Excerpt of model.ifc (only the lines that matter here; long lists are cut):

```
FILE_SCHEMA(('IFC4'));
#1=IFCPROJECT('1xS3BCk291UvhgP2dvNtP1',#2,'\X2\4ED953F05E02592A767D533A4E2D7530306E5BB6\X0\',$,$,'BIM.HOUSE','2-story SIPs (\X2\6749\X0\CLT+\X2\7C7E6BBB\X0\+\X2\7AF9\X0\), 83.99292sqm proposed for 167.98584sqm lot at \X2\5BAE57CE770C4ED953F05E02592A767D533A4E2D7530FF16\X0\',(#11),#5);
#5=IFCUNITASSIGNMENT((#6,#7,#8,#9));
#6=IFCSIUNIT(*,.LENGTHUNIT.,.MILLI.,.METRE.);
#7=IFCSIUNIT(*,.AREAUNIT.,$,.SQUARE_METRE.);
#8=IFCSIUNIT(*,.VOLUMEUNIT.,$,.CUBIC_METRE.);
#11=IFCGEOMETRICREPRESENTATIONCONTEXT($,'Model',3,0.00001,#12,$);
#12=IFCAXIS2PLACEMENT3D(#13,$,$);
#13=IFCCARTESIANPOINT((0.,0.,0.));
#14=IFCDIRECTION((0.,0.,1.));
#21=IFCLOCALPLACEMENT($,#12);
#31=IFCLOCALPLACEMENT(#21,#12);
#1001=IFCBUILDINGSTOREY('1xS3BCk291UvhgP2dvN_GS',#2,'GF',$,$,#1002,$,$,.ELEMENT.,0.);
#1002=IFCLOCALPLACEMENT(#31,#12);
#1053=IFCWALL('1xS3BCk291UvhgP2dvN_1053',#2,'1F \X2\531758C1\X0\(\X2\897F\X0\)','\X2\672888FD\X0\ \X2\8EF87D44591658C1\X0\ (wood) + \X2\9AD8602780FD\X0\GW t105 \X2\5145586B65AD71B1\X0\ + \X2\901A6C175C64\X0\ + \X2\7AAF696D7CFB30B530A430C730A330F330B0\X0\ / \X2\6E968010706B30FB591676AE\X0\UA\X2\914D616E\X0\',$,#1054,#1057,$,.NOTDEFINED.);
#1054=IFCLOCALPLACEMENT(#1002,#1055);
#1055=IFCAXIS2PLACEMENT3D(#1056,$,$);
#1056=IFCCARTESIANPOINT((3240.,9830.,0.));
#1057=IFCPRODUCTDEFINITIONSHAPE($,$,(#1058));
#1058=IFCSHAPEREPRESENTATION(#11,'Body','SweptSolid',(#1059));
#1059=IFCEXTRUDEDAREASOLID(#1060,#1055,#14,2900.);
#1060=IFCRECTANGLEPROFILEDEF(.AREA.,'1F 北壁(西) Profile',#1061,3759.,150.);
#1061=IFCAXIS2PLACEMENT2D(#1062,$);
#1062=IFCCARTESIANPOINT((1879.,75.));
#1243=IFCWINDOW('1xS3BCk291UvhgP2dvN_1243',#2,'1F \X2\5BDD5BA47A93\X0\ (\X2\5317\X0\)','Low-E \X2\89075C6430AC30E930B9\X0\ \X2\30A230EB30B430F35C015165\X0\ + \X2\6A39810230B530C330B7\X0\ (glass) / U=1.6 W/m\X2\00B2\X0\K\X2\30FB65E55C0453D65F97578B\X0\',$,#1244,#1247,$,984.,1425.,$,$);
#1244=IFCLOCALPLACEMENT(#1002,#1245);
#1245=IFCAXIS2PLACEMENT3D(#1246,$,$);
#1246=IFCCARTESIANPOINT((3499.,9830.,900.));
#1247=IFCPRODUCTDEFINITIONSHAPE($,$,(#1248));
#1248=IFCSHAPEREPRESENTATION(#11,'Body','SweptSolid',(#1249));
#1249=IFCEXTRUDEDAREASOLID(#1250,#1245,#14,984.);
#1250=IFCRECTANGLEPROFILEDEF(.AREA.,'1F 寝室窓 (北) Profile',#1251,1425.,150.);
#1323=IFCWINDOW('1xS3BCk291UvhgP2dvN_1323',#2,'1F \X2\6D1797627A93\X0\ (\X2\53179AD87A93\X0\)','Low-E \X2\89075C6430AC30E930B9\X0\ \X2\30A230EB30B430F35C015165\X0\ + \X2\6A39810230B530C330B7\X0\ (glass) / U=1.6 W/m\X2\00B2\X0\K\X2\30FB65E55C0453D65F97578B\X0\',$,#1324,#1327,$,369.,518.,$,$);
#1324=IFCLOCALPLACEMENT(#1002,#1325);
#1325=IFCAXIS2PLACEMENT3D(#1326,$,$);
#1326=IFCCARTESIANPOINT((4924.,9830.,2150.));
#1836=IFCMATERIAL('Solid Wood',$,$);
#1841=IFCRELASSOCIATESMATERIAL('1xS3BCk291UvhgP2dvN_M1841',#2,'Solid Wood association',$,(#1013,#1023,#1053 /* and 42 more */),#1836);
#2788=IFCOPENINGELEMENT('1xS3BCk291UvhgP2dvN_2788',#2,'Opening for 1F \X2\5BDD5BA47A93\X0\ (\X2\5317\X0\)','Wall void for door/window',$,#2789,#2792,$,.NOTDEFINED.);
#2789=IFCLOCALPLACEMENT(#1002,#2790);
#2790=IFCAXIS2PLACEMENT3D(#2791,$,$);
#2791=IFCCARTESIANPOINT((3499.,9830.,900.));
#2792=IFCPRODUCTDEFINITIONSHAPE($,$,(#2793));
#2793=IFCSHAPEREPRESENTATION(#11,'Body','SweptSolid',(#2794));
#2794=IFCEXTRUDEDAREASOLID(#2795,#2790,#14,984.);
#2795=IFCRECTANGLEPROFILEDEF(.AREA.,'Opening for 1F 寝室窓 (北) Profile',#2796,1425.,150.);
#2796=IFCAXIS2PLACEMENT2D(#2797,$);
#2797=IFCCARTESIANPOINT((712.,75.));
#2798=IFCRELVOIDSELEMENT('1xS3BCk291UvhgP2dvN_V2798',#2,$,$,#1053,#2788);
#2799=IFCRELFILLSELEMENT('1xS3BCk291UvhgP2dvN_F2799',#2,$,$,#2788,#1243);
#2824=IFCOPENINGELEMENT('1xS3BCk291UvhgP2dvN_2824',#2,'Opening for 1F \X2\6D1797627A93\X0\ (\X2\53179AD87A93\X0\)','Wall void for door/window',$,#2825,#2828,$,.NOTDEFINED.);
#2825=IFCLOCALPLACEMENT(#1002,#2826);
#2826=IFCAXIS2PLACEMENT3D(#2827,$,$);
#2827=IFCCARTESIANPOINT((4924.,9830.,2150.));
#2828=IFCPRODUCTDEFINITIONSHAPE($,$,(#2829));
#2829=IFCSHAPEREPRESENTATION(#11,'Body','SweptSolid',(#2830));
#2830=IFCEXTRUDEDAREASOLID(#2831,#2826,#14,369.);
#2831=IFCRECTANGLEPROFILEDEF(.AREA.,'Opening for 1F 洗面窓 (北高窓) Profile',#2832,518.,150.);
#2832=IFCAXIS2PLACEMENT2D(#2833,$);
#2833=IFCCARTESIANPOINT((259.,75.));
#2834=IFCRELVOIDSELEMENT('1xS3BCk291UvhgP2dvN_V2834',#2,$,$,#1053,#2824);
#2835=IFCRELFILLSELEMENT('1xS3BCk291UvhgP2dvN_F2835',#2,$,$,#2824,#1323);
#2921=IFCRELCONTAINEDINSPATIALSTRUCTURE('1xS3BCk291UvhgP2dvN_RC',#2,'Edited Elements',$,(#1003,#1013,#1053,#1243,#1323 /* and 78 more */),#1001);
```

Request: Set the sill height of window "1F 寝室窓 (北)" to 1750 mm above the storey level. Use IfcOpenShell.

```python
import numpy as np
import ifcopenshell
import ifcopenshell.api.geometry
import ifcopenshell.geom
import ifcopenshell.util.element
import ifcopenshell.util.placement
import ifcopenshell.util.shape
import ifcopenshell.util.unit

model = ifcopenshell.open("model.ifc")
unit_scale = ifcopenshell.util.unit.calculate_unit_scale(model)

window = model.by_guid("1xS3BCk291UvhgP2dvN_1243")
opening = window.FillsVoids[0].RelatingOpeningElement
storey = ifcopenshell.util.element.get_container(window, ifc_class="IfcBuildingStorey")
level = ifcopenshell.util.placement.get_local_placement(storey.ObjectPlacement)[2, 3]

# The opening's origin need not be at the sill, so measure its lowest point.
shape = ifcopenshell.geom.create_shape(ifcopenshell.geom.settings(), opening)
bottom = ifcopenshell.util.shape.get_shape_bottom_elevation(shape, shape.geometry) / unit_scale
dz = level + 1.75 / unit_scale - bottom

shift = np.array([0.0, 0.0, dz])
# The window is not placed relative to its opening, so move both.
for product in (opening, window):
    matrix = ifcopenshell.util.placement.get_local_placement(product.ObjectPlacement)
    matrix[:3, 3] += shift
    ifcopenshell.api.geometry.edit_object_placement(model, product=product, matrix=matrix, is_si=False)

print(f"moved by {dz * unit_scale:+.3f} m")

model.write("model_rev.ifc")
```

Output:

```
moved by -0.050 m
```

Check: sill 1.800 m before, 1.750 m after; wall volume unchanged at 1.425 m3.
